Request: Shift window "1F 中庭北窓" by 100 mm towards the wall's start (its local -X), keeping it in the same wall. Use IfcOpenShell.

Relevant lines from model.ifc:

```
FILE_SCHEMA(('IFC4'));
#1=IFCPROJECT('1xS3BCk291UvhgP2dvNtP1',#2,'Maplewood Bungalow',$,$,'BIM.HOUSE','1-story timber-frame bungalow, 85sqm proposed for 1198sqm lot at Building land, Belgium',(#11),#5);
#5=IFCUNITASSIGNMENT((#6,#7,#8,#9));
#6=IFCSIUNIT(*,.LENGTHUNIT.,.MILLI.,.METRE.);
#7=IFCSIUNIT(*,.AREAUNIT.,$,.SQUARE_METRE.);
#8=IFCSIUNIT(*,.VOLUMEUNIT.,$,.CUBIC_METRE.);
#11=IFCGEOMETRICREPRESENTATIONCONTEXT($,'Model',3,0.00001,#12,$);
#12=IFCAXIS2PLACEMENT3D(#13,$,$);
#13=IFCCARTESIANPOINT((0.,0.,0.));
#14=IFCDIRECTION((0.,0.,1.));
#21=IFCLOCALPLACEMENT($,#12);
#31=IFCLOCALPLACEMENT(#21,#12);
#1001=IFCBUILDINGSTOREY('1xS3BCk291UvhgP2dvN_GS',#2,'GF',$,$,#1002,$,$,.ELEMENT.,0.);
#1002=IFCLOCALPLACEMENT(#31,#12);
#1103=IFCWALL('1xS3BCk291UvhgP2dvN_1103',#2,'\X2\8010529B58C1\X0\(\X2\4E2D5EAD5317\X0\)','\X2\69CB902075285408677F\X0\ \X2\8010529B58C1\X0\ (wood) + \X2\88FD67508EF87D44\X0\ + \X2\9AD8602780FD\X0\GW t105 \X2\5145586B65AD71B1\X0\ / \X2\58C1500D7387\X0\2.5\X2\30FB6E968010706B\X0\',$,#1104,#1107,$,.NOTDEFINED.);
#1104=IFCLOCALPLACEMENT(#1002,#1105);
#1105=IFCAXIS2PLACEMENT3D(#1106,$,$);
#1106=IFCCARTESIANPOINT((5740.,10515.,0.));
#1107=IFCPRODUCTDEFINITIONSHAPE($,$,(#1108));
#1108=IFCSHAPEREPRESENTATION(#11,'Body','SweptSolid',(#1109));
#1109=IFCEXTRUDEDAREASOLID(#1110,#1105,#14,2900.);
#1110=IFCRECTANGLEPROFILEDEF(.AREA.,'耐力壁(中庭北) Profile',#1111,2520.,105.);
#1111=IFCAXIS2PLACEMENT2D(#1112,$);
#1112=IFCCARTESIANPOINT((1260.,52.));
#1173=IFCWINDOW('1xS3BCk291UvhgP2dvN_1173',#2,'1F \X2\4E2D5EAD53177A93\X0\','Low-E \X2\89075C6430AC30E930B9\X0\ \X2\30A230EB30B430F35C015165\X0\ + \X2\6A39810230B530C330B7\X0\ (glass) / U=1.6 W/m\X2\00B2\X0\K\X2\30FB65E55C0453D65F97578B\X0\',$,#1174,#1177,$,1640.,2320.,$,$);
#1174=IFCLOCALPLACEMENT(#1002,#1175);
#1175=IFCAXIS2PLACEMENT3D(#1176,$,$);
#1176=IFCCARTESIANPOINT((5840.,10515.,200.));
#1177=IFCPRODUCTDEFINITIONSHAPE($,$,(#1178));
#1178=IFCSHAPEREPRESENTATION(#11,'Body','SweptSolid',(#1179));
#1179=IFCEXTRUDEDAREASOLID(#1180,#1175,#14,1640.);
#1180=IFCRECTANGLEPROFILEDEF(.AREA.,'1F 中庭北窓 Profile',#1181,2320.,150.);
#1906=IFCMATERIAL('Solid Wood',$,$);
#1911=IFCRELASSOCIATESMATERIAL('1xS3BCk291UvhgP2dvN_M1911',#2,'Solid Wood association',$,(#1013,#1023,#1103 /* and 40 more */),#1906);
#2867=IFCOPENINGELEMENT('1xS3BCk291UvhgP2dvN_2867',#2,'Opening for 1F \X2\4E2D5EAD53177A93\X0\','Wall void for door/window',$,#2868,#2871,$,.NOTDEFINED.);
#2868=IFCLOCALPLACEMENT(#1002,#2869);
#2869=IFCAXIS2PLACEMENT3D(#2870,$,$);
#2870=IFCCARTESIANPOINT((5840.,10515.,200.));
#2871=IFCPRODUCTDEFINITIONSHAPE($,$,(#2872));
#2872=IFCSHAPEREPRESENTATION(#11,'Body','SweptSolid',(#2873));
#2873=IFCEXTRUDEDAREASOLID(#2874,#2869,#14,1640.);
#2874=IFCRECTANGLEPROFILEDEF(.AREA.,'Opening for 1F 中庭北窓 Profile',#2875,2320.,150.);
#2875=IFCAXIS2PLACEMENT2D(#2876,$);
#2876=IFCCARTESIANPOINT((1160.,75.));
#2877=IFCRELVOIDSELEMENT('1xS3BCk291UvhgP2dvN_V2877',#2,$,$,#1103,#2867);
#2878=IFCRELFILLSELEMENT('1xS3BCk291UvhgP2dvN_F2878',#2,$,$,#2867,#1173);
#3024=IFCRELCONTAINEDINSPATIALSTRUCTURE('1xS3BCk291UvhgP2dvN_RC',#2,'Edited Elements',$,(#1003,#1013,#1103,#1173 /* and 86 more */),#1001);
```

```python
import ifcopenshell
import ifcopenshell.api.geometry
import ifcopenshell.util.placement
import ifcopenshell.util.unit

model = ifcopenshell.open("model.ifc")
unit_scale = ifcopenshell.util.unit.calculate_unit_scale(model)

window = model.by_guid("1xS3BCk291UvhgP2dvN_1173")
opening = window.FillsVoids[0].RelatingOpeningElement
wall = opening.VoidsElements[0].RelatingBuildingElement

wall_matrix = ifcopenshell.util.placement.get_local_placement(wall.ObjectPlacement)
shift = wall_matrix[:3, 0] * -0.1 / unit_scale
before = ifcopenshell.util.placement.get_local_placement(window.ObjectPlacement)[:3, 3].copy()

# The window is not placed relative to its opening, so move both.
for product in (opening, window):
    matrix = ifcopenshell.util.placement.get_local_placement(product.ObjectPlacement)
    matrix[:3, 3] += shift
    ifcopenshell.api.geometry.edit_object_placement(model, product=product, matrix=matrix, is_si=False)

after = ifcopenshell.util.placement.get_local_placement(window.ObjectPlacement)[:3, 3]
print("window moved by", (after - before).round(3) + 0.0)

model.write("model_updated.ifc")
```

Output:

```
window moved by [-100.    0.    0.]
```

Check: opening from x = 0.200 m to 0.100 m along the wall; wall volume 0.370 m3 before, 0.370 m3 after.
